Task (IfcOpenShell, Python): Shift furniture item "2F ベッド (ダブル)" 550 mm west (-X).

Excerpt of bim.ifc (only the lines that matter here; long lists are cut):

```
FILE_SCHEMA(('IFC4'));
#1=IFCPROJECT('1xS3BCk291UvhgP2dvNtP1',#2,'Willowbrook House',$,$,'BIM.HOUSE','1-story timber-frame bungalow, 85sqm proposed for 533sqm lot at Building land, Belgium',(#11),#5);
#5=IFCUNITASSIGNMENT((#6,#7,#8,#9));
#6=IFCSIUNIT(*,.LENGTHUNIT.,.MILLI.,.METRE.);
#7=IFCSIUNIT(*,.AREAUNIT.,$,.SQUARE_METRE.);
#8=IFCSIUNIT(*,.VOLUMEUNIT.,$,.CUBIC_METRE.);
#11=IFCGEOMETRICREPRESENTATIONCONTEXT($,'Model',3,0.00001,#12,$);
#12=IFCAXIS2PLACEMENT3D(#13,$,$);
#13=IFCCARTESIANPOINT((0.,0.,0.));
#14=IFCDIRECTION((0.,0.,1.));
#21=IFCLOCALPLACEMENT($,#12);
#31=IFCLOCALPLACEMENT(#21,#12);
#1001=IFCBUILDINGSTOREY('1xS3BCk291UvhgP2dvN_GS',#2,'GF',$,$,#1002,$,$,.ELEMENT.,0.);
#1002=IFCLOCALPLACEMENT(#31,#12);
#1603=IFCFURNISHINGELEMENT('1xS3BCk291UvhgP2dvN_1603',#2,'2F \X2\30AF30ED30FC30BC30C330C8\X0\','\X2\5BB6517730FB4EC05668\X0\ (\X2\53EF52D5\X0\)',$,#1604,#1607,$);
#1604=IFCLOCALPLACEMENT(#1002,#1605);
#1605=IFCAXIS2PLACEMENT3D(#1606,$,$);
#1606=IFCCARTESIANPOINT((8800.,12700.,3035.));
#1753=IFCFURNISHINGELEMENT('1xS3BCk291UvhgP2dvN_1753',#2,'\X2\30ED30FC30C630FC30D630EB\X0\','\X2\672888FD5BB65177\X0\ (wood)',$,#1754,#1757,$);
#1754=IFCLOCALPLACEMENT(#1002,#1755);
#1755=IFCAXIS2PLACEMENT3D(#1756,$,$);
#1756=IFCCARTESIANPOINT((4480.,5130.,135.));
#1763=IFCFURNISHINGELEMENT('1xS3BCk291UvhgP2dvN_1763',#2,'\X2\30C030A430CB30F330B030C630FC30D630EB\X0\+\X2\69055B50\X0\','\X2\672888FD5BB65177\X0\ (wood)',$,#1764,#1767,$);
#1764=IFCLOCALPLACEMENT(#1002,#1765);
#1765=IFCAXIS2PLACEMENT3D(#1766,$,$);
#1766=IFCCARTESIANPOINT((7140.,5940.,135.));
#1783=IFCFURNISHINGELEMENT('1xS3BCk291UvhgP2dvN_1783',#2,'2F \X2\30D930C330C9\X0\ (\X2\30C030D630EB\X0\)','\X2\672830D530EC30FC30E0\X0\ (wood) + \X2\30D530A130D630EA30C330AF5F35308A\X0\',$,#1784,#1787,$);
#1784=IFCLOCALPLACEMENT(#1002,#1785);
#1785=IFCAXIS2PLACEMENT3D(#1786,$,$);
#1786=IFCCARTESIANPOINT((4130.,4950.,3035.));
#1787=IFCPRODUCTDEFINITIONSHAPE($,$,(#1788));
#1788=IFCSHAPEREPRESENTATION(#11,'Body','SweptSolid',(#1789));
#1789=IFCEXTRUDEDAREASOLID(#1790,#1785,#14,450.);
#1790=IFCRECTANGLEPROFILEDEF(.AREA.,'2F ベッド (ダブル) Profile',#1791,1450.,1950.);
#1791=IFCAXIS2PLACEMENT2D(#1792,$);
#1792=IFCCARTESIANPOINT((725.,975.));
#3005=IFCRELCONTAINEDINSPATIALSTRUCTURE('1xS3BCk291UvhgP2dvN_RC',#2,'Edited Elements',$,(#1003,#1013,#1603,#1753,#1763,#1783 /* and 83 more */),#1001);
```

```python
import ifcopenshell
import ifcopenshell.api.geometry
import ifcopenshell.util.placement
import ifcopenshell.util.unit

model = ifcopenshell.open("bim.ifc")
unit_scale = ifcopenshell.util.unit.calculate_unit_scale(model)

item = model.by_id(1783)
matrix = ifcopenshell.util.placement.get_local_placement(item.ObjectPlacement)
matrix[0, 3] -= 0.55 / unit_scale
ifcopenshell.api.geometry.edit_object_placement(model, product=item, matrix=matrix, is_si=False)

print(ifcopenshell.util.placement.get_local_placement(item.ObjectPlacement).round(3) + 0.0)

model.write("bim_updated.ifc")
```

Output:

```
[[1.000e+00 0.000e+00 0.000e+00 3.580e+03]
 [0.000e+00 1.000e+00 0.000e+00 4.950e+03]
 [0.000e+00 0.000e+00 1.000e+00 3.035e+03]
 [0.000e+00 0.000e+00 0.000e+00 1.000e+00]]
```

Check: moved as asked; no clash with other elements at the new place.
